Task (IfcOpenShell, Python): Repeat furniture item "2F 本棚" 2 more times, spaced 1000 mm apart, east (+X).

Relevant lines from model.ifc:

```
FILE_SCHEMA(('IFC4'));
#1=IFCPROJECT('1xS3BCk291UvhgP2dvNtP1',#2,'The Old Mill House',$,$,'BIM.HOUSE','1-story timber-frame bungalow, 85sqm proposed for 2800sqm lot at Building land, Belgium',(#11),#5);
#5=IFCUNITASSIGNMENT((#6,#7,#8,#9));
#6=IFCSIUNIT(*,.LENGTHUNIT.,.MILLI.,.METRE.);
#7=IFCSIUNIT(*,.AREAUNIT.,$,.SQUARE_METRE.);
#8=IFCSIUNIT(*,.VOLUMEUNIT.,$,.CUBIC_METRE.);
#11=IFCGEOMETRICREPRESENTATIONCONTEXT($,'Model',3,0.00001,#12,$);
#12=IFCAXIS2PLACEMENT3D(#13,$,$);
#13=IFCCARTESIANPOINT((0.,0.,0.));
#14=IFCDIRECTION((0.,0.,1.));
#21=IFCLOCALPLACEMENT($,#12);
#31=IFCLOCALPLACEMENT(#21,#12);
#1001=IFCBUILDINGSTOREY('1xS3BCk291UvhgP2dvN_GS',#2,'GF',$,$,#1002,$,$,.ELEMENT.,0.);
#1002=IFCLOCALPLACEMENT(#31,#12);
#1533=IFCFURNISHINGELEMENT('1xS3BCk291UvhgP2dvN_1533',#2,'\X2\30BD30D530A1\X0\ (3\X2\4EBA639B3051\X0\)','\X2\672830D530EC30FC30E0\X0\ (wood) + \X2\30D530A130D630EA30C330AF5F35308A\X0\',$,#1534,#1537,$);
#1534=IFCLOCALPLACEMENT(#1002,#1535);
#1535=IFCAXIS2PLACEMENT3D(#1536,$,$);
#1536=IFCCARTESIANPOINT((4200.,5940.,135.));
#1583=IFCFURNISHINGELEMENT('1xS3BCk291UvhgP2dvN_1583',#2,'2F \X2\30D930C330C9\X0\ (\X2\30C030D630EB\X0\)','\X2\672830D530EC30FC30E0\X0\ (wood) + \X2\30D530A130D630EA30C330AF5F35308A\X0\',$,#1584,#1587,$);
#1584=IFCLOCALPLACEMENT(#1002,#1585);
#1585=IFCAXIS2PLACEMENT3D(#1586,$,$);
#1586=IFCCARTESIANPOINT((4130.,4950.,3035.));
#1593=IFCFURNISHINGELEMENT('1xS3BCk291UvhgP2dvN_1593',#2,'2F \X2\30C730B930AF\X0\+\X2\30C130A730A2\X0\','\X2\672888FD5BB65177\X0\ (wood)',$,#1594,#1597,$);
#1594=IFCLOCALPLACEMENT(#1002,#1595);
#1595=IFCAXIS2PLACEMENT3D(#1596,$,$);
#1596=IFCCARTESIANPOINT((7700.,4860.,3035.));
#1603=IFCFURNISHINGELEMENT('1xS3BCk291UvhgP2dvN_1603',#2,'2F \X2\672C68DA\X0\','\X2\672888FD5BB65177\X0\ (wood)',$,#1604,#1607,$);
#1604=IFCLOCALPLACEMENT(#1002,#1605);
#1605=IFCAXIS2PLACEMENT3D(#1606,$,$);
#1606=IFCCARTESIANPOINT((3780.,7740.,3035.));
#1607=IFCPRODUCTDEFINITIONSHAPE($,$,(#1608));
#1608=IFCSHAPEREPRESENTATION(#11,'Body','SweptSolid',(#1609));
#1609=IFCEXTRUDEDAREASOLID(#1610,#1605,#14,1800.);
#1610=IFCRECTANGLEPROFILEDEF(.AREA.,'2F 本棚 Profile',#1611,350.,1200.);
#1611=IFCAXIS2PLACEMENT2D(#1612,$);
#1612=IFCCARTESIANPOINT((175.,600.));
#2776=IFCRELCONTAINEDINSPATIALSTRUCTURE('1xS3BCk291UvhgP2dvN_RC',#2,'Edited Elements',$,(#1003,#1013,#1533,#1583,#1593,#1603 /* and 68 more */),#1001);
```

```python
import numpy as np
import ifcopenshell
import ifcopenshell.api.geometry
import ifcopenshell.api.root
import ifcopenshell.util.element
import ifcopenshell.util.placement
import ifcopenshell.util.unit

model = ifcopenshell.open("model.ifc")
unit_scale = ifcopenshell.util.unit.calculate_unit_scale(model)


def reuse_history(source, copy):
    """copy_class also copies each property set's owner history, people and application; keep the originals."""
    for rel in copy.IsDefinedBy:
        if rel.is_a("IfcRelDefinesByProperties") and (history := rel.RelatingPropertyDefinition.OwnerHistory):
            rel.RelatingPropertyDefinition.OwnerHistory = source.OwnerHistory
            ifcopenshell.util.element.remove_deep2(model, history)


source = model.by_guid("1xS3BCk291UvhgP2dvN_1603")
base = ifcopenshell.util.placement.get_local_placement(source.ObjectPlacement)
step = np.array([1.0, 0.0, 0.0]) * 1 / unit_scale

for i in range(1, 3):
    copy = ifcopenshell.api.root.copy_class(model, product=source)
    copy.Representation = ifcopenshell.util.element.copy_deep(
        model, source.Representation, exclude=["IfcGeometricRepresentationContext", "IfcRepresentationMap"]
    )
    reuse_history(source, copy)
    matrix = base.copy()
    matrix[:3, 3] += i * step
    print("added at", matrix[:3, 3].round(3) + 0.0)
    ifcopenshell.api.geometry.edit_object_placement(model, product=copy, matrix=matrix, is_si=False)

model.write("model_edited.ifc")
```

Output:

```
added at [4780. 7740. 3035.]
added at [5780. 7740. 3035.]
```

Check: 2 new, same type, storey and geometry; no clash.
